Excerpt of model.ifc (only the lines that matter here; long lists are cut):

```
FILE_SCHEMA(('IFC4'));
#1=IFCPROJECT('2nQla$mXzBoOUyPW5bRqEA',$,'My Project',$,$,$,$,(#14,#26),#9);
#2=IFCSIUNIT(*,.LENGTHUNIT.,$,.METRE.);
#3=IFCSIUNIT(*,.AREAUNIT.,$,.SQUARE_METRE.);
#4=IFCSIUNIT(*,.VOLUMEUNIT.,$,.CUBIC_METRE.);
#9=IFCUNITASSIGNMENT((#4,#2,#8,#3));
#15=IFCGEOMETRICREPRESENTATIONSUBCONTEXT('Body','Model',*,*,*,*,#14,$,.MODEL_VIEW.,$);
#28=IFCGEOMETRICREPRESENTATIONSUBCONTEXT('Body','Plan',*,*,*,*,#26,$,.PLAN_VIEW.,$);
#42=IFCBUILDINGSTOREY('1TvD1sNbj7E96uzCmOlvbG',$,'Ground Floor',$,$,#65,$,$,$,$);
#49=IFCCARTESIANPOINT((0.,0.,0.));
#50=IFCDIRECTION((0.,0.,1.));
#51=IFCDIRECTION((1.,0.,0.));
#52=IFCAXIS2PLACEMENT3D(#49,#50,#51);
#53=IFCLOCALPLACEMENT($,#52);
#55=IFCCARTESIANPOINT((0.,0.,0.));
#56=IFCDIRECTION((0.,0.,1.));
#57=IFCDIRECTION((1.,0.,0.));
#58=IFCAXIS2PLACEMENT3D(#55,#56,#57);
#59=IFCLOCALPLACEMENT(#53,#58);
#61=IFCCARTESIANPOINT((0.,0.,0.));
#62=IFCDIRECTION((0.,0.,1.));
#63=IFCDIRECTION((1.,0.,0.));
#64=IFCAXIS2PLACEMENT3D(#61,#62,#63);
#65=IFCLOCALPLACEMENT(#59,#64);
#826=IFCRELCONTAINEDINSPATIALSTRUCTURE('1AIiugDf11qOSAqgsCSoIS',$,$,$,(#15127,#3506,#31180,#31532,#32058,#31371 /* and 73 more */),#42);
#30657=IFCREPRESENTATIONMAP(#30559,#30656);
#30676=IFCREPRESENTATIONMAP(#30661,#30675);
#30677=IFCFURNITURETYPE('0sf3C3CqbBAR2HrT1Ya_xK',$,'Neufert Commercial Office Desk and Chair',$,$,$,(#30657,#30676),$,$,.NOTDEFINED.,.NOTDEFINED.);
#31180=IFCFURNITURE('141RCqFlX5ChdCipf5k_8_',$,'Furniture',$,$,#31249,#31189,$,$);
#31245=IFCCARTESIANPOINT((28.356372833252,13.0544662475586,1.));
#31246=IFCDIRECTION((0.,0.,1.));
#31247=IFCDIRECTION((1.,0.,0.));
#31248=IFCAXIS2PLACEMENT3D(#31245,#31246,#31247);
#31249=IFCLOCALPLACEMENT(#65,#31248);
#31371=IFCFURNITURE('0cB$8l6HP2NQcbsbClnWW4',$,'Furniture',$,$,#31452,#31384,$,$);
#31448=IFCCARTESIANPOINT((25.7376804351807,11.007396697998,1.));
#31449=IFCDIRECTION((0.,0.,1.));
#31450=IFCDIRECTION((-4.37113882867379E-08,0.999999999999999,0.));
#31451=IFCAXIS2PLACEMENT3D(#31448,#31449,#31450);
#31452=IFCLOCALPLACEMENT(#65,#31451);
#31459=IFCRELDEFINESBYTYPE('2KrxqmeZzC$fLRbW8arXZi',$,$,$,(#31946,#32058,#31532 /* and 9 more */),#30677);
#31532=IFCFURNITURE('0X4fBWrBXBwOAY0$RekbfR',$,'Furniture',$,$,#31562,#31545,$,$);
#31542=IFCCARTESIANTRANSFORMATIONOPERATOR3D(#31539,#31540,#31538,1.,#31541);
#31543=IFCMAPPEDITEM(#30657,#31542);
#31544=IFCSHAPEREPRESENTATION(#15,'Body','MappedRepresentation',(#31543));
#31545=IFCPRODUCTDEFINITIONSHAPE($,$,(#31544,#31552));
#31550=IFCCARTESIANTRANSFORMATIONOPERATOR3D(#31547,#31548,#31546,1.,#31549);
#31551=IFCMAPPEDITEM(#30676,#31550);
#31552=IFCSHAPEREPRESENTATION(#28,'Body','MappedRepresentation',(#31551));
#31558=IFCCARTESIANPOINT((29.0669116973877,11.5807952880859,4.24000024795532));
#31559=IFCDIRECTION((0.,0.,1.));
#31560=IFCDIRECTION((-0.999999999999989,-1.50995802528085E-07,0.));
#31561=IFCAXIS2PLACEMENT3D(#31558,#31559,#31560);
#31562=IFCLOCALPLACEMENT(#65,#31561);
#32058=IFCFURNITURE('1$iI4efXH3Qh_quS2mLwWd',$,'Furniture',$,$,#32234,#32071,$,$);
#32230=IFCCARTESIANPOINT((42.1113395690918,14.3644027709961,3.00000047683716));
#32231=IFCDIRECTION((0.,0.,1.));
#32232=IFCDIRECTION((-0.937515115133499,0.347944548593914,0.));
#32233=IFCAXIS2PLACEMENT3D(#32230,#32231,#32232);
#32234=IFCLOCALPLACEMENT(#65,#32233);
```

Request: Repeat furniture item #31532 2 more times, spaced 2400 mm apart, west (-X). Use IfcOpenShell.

```python
import numpy as np
import ifcopenshell
import ifcopenshell.api.geometry
import ifcopenshell.api.root
import ifcopenshell.util.element
import ifcopenshell.util.placement
import ifcopenshell.util.unit

model = ifcopenshell.open("model.ifc")
unit_scale = ifcopenshell.util.unit.calculate_unit_scale(model)

source = model.by_guid("0X4fBWrBXBwOAY0$RekbfR")
base = ifcopenshell.util.placement.get_local_placement(source.ObjectPlacement)
step = np.array([-1.0, 0.0, 0.0]) * 2.4 / unit_scale

for i in range(1, 3):
    copy = ifcopenshell.api.root.copy_class(model, product=source)
    copy.Representation = ifcopenshell.util.element.copy_deep(
        model, source.Representation, exclude=["IfcGeometricRepresentationContext", "IfcRepresentationMap"]
    )
    matrix = base.copy()
    matrix[:3, 3] += i * step
    print("added at", matrix[:3, 3].round(3) + 0.0)
    ifcopenshell.api.geometry.edit_object_placement(model, product=copy, matrix=matrix, is_si=False)

model.write("model_edited.ifc")
```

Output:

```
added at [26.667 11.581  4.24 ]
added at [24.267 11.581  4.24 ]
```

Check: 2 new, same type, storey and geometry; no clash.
